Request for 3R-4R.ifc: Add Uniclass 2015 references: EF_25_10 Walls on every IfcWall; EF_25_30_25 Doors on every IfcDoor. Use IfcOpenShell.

First a look at what the model holds.

```python
import ifcopenshell

model = ifcopenshell.open("3R-4R.ifc")
print(model.schema)
print("classifications:", [c.Name for c in model.by_type("IfcClassification")])
for ifc_class in ("IfcDoor", "IfcRoof", "IfcStair", "IfcWall", "IfcWindow"):
    print(ifc_class, len(model.by_type(ifc_class)))
```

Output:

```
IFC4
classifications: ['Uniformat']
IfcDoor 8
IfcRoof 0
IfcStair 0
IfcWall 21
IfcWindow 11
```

```python
import ifcopenshell
import ifcopenshell.api.classification

model = ifcopenshell.open("3R-4R.ifc")

system = ifcopenshell.api.classification.add_classification(model, classification="Uniclass 2015")

codes = {
    "IfcWall": ("EF_25_10", "Walls"),
    "IfcDoor": ("EF_25_30_25", "Doors"),
}
for ifc_class, (code, name) in codes.items():
    products = model.by_type(ifc_class)
    ifcopenshell.api.classification.add_reference(
        model, products=products, classification=system, identification=code, name=name
    )
    print(code, len(products))

model.write("3R-4R_rev.ifc")
```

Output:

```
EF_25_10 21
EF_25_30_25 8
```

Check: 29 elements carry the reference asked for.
